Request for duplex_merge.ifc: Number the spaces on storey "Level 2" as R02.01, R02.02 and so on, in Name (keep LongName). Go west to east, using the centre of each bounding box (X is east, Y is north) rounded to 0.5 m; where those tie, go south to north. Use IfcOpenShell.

First a look at what the model holds.

```python
import ifcopenshell
import ifcopenshell.util.element
import ifcopenshell.util.placement

model = ifcopenshell.open("duplex_merge.ifc")
print(model.schema)
storey = next(s for s in model.by_type("IfcBuildingStorey") if s.Name == "Level 2")
spaces = [e for e in ifcopenshell.util.element.get_decomposition(storey) if e.is_a("IfcSpace")]
for e in sorted(spaces, key=lambda e: e.id()):
    origin = ifcopenshell.util.placement.get_local_placement(e.ObjectPlacement)[:3, 3]
    print(e.id(), e.Name, e.LongName, origin.round(2) + 0.0, sep=" | ")
```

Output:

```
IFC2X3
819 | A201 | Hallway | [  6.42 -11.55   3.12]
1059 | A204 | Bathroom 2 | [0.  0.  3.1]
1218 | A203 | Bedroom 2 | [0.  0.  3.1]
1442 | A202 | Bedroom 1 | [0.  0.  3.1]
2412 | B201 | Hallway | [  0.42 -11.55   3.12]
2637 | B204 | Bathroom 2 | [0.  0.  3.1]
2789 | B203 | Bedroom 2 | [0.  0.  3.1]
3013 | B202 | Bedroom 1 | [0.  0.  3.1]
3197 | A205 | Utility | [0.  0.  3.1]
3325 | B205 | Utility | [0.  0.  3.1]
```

```python
import ifcopenshell
import ifcopenshell.geom
import ifcopenshell.util.element
import ifcopenshell.util.shape

model = ifcopenshell.open("duplex_merge.ifc")
settings = ifcopenshell.geom.settings()
settings.set("use-world-coords", True)


def centre(element):
    shape = ifcopenshell.geom.create_shape(settings, element)
    return ifcopenshell.util.shape.get_bbox_centroid(shape.geometry)


storey = next(s for s in model.by_type("IfcBuildingStorey") if s.Name == "Level 2")
spaces = [e for e in ifcopenshell.util.element.get_decomposition(storey) if e.is_a("IfcSpace")]

# Insertion points can sit at a corner or the storey origin, so sort by the geometry (in metres).
centres = {e: centre(e) for e in spaces}
spaces.sort(key=lambda e: (round(centres[e][0] / 0.5), centres[e][1]))

for i, e in enumerate(spaces, start=1):
    number = f"R02.{i:02d}"
    e.Name = number
    print(e.id(), number)

model.write("duplex_merge-out.ifc")
```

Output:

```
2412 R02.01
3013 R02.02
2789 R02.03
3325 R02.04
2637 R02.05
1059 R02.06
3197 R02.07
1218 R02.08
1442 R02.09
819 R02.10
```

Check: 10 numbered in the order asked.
